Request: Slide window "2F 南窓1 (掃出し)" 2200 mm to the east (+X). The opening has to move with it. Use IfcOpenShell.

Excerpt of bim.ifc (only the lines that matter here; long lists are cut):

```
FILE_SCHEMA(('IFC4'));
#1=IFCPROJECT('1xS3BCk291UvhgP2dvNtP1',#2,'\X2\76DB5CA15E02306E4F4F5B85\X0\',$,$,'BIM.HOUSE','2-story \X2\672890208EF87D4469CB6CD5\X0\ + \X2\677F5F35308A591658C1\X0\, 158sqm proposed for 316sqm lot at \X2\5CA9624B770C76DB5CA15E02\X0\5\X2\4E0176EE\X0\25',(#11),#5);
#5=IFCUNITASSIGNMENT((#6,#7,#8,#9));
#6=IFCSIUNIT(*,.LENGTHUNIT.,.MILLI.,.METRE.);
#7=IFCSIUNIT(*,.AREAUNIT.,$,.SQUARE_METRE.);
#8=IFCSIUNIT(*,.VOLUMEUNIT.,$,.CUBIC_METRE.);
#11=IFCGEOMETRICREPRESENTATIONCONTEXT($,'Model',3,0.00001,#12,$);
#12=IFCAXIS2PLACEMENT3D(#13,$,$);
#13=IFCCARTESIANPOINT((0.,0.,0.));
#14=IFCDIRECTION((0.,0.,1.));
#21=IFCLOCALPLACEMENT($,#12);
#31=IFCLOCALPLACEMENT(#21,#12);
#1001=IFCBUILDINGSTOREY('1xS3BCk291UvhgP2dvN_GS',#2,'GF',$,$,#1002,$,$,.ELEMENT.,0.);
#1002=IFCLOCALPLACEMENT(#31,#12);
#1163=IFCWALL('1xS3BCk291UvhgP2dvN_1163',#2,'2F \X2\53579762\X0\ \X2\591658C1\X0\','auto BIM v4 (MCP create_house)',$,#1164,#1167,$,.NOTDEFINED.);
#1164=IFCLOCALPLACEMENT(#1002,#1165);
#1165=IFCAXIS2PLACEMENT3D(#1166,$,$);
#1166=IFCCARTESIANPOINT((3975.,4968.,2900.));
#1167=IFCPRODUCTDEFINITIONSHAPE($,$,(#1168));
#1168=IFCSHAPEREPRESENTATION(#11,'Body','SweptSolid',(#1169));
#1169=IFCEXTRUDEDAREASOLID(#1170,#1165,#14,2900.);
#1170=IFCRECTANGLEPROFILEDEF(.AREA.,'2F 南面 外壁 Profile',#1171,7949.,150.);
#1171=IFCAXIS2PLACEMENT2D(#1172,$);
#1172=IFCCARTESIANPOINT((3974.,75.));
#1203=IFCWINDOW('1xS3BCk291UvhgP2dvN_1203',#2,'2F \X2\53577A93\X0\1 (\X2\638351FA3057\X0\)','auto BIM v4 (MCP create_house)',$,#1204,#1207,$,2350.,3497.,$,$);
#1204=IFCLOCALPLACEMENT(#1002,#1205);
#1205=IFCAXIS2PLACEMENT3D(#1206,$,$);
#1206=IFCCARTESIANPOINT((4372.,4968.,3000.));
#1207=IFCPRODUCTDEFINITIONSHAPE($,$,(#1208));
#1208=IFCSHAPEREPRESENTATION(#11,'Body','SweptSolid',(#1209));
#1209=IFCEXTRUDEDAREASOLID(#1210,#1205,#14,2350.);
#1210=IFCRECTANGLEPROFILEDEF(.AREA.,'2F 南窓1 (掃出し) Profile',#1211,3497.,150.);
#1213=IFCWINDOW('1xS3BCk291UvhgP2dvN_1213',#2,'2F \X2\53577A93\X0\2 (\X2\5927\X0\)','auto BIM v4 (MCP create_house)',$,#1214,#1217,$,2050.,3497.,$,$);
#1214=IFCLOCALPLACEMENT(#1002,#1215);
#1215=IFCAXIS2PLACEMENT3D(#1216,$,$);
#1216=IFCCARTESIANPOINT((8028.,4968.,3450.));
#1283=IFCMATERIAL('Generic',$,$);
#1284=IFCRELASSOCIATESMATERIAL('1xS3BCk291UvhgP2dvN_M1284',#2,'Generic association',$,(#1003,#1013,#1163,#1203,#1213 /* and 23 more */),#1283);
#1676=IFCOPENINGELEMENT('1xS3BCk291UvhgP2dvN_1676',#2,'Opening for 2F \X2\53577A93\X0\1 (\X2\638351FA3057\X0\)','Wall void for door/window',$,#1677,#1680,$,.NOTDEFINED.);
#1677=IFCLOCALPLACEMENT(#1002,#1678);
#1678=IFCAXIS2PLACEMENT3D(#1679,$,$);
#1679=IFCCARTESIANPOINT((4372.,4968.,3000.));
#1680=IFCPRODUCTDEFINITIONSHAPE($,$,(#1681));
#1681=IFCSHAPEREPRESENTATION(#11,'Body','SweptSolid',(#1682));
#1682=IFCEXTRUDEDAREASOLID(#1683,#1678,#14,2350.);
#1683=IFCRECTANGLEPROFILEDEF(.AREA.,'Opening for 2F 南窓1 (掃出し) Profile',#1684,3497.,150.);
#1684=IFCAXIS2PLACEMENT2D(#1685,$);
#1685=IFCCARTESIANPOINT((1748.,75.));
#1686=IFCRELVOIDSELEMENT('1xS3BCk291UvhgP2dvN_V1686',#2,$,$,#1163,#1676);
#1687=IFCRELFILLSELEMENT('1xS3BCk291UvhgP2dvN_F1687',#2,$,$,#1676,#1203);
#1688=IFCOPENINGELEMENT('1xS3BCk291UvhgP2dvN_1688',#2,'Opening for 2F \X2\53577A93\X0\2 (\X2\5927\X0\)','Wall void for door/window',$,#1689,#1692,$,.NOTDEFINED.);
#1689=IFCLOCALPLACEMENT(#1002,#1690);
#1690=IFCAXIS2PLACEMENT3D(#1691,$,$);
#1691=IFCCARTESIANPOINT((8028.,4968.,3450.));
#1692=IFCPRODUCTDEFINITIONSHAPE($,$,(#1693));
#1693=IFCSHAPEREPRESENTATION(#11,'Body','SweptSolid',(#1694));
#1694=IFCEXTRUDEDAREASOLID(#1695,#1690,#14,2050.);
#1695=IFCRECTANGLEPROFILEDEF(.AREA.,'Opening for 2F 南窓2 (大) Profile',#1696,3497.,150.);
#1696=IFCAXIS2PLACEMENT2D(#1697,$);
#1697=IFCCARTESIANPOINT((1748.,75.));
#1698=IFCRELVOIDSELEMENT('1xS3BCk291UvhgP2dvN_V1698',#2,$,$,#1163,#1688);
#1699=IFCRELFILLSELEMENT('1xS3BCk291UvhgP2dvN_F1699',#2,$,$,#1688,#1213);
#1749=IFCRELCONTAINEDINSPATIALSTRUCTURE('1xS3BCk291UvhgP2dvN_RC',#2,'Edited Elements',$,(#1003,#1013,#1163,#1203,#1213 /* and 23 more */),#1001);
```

```python
import ifcopenshell
import ifcopenshell.api.geometry
import ifcopenshell.util.placement
import ifcopenshell.util.unit

model = ifcopenshell.open("bim.ifc")
unit_scale = ifcopenshell.util.unit.calculate_unit_scale(model)

window = model.by_guid("1xS3BCk291UvhgP2dvN_1203")
opening = window.FillsVoids[0].RelatingOpeningElement
wall = opening.VoidsElements[0].RelatingBuildingElement

wall_matrix = ifcopenshell.util.placement.get_local_placement(wall.ObjectPlacement)
shift = wall_matrix[:3, 0] * 2.2 / unit_scale
before = ifcopenshell.util.placement.get_local_placement(window.ObjectPlacement)[:3, 3].copy()

# The window is not placed relative to its opening, so move both.
for product in (opening, window):
    matrix = ifcopenshell.util.placement.get_local_placement(product.ObjectPlacement)
    matrix[:3, 3] += shift
    ifcopenshell.api.geometry.edit_object_placement(model, product=product, matrix=matrix, is_si=False)

after = ifcopenshell.util.placement.get_local_placement(window.ObjectPlacement)[:3, 3]
print("window moved by", (after - before).round(3) + 0.0)

model.write("bim_rev.ifc")
```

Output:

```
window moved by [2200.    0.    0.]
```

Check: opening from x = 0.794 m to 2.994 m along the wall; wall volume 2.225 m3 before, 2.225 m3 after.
